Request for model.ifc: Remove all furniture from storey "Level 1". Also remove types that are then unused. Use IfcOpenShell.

First a look at what the model holds.

```python
import ifcopenshell
import ifcopenshell.util.element

model = ifcopenshell.open("model.ifc")
print(model.schema)
storey = next(s for s in model.by_type("IfcBuildingStorey") if s.Name == "Level 1")
furniture = [e for e in ifcopenshell.util.element.get_decomposition(storey) if e.is_a("IfcFurnishingElement")]
seen = {}
for e in furniture:
    element_type = ifcopenshell.util.element.get_type(e)
    name = element_type.Name if element_type not in (None, e) else None
    seen[name] = seen.get(name, 0) + 1
for name, count in sorted(seen.items(), key=str):
    print(count, "x", name)
```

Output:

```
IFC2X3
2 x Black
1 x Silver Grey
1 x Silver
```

```python
import ifcopenshell
import ifcopenshell.api.root
import ifcopenshell.util.element

model = ifcopenshell.open("model.ifc")

storey = next(s for s in model.by_type("IfcBuildingStorey") if s.Name == "Level 1")
furniture = [e for e in ifcopenshell.util.element.get_decomposition(storey) if e.is_a("IfcFurnishingElement")]
types = {ifcopenshell.util.element.get_type(e) for e in furniture} - {None, *furniture}

for e in furniture:
    ifcopenshell.api.root.remove_product(model, product=e)
print(len(furniture), "removed")

unused = [t for t in types if not ifcopenshell.util.element.get_types(t)]
for t in unused:
    ifcopenshell.api.root.remove_product(model, product=t)
print(len(unused), "unused types removed")

model.write("model_edited.ifc")
```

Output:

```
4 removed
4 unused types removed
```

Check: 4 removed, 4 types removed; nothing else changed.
